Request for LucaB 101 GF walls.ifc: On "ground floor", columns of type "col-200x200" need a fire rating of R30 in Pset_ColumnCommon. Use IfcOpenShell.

First a look at what the model holds.

```python
import ifcopenshell
import ifcopenshell.util.element

model = ifcopenshell.open("LucaB 101 GF walls.ifc")
print(model.schema)
storey = next(s for s in model.by_type("IfcBuildingStorey") if s.Name == "ground floor")
columns = [e for e in ifcopenshell.util.element.get_decomposition(storey) if e.is_a("IfcColumn")]
seen = {}
for e in columns:
    element_type = ifcopenshell.util.element.get_type(e)
    key = (element_type.Name if element_type != e and element_type else None, ifcopenshell.util.element.get_pset(e, "Pset_ColumnCommon", "FireRating"))
    seen[key] = seen.get(key, 0) + 1
for (name, value), count in sorted(seen.items(), key=str):
    print(count, "x", name, "|", value)
```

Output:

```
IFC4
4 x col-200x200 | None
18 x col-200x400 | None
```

```python
import ifcopenshell
import ifcopenshell.api.pset
import ifcopenshell.util.element

model = ifcopenshell.open("LucaB 101 GF walls.ifc")

storey = next(s for s in model.by_type("IfcBuildingStorey") if s.Name == "ground floor")
columns = [e for e in ifcopenshell.util.element.get_decomposition(storey) if e.is_a("IfcColumn")]

count = 0
for e in columns:
    element_type = ifcopenshell.util.element.get_type(e)
    if element_type in (None, e) or element_type.Name != "col-200x200":
        continue
    # add_pset returns the element's existing set when there is one.
    pset = ifcopenshell.api.pset.add_pset(model, product=e, name="Pset_ColumnCommon")
    ifcopenshell.api.pset.edit_pset(model, pset=pset, properties={"FireRating": "R30"})
    count += 1

print(count, "columns updated")

model.write("LucaB 101 GF walls_v2.ifc")
```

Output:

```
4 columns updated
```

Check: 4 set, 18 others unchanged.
